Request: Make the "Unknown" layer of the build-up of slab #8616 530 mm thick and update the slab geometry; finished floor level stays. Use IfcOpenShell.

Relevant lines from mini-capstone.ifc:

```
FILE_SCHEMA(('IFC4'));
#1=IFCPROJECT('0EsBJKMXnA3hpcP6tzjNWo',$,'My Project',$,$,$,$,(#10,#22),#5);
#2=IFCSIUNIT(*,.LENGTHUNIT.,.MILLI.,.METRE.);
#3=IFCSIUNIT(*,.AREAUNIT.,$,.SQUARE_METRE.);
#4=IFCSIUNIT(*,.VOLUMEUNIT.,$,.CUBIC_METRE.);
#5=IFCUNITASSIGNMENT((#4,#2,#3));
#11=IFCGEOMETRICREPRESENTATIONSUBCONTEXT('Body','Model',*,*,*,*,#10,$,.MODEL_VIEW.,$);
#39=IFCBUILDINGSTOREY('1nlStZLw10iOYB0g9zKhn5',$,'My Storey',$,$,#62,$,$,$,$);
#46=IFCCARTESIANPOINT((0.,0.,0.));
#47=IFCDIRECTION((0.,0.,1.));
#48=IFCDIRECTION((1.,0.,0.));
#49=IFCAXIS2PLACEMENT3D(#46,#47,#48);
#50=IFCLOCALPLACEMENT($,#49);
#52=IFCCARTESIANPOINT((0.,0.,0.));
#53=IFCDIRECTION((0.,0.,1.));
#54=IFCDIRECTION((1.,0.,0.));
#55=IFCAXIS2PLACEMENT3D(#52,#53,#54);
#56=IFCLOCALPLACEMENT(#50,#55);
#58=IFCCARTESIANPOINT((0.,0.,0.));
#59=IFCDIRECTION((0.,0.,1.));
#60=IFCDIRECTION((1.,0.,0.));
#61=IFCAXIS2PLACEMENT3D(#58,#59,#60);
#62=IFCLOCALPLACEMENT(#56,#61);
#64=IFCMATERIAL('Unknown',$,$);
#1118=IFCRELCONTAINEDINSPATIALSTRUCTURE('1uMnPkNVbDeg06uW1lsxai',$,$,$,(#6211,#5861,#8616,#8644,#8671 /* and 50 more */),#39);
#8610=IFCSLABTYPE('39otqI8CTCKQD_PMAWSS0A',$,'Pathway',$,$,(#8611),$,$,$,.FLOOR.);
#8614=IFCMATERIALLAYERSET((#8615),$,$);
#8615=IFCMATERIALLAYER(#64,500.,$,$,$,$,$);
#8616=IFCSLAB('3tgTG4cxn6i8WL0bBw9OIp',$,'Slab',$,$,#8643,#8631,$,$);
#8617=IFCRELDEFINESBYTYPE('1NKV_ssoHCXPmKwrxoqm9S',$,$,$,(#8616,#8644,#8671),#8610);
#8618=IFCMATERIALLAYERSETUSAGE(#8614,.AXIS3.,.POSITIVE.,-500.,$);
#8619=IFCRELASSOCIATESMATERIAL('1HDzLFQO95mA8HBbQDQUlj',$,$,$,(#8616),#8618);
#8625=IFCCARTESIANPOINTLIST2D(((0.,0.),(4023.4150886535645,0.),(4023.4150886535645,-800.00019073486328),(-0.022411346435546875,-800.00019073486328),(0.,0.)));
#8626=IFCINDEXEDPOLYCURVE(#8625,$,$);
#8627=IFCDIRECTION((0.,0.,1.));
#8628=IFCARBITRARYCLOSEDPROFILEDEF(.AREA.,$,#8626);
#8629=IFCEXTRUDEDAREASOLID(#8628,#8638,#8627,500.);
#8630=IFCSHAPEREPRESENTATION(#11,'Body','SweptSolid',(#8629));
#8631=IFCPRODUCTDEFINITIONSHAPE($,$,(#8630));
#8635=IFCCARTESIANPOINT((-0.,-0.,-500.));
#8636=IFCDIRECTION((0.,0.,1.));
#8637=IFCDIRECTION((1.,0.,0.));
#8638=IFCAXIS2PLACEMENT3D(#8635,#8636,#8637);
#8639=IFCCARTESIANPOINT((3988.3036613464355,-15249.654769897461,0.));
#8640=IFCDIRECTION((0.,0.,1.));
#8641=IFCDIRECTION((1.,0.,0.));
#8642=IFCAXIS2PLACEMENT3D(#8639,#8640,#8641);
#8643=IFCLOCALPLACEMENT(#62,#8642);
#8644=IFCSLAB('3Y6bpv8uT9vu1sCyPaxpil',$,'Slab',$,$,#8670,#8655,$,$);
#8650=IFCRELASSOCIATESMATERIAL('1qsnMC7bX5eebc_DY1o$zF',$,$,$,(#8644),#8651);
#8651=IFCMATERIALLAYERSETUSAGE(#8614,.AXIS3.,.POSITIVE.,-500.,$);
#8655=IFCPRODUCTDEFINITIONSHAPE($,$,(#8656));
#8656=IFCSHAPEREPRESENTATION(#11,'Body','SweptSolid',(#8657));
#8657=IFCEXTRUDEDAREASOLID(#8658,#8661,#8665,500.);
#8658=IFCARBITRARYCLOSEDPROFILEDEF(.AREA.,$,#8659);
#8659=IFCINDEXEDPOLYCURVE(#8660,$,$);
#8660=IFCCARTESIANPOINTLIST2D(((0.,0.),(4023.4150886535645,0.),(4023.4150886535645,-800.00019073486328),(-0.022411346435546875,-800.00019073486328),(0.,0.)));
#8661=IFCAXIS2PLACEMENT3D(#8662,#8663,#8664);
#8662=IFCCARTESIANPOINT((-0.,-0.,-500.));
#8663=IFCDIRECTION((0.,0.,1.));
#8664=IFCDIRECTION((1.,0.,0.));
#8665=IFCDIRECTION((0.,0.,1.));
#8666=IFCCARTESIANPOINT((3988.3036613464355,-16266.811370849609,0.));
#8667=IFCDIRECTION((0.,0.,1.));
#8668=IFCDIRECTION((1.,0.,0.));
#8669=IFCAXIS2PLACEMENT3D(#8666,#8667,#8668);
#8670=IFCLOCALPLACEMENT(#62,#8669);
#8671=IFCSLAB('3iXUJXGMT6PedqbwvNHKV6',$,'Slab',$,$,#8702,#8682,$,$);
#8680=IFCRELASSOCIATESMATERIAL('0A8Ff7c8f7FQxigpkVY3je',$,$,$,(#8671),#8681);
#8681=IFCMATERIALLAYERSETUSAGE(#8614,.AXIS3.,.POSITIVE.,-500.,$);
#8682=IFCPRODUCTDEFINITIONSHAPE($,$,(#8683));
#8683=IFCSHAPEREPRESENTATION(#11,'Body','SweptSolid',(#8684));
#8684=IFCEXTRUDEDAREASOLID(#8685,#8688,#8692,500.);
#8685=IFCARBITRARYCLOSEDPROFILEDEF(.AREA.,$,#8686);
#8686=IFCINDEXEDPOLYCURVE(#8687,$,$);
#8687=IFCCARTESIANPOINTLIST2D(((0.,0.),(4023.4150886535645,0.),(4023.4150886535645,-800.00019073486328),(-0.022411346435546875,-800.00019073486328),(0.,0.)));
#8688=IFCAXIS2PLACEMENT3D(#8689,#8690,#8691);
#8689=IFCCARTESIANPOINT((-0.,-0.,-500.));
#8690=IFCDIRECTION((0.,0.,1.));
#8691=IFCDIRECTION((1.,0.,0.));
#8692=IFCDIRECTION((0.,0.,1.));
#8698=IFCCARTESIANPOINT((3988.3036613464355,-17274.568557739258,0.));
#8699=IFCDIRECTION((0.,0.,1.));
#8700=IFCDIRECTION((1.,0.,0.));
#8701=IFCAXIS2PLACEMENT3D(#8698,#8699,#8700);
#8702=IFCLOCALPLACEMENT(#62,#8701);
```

```python
import ifcopenshell
import ifcopenshell.util.element
import ifcopenshell.util.representation
import ifcopenshell.util.unit

model = ifcopenshell.open("mini-capstone.ifc")
unit_scale = ifcopenshell.util.unit.calculate_unit_scale(model)

layer_set = model.by_id(8614)
layer = next(l for l in layer_set.MaterialLayers if l.Material and l.Material.Name == "Unknown")
change = 0.53 / unit_scale - layer.LayerThickness
layer.LayerThickness += change

# The layer set is shared, so every slab that uses it gets the new thickness.
slabs = [e for e in ifcopenshell.util.element.get_elements_by_material(model, layer_set) if e.is_a("IfcSlab")]
for slab in sorted(slabs, key=lambda e: e.id()):
    body = ifcopenshell.util.representation.get_representation(slab, "Model", "Body")
    solid = body.Items[0]
    old_depth = solid.Depth
    solid.Depth += change
    # Extruded upwards: lower the start of the extrusion so the top stays.
    x, y, z = solid.Position.Location.Coordinates
    solid.Position.Location = model.createIfcCartesianPoint((x, y, z - change))
    print(slab.id(), f"{old_depth:g} -> {solid.Depth:g}")

# The layers are counted up from the underside, which has moved.
for usage in {ifcopenshell.util.element.get_material(slab) for slab in slabs}:
    usage.OffsetFromReferenceLine -= change

model.write("mini-capstone_v2.ifc")
```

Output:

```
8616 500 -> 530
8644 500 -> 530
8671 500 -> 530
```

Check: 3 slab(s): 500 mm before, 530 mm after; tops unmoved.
